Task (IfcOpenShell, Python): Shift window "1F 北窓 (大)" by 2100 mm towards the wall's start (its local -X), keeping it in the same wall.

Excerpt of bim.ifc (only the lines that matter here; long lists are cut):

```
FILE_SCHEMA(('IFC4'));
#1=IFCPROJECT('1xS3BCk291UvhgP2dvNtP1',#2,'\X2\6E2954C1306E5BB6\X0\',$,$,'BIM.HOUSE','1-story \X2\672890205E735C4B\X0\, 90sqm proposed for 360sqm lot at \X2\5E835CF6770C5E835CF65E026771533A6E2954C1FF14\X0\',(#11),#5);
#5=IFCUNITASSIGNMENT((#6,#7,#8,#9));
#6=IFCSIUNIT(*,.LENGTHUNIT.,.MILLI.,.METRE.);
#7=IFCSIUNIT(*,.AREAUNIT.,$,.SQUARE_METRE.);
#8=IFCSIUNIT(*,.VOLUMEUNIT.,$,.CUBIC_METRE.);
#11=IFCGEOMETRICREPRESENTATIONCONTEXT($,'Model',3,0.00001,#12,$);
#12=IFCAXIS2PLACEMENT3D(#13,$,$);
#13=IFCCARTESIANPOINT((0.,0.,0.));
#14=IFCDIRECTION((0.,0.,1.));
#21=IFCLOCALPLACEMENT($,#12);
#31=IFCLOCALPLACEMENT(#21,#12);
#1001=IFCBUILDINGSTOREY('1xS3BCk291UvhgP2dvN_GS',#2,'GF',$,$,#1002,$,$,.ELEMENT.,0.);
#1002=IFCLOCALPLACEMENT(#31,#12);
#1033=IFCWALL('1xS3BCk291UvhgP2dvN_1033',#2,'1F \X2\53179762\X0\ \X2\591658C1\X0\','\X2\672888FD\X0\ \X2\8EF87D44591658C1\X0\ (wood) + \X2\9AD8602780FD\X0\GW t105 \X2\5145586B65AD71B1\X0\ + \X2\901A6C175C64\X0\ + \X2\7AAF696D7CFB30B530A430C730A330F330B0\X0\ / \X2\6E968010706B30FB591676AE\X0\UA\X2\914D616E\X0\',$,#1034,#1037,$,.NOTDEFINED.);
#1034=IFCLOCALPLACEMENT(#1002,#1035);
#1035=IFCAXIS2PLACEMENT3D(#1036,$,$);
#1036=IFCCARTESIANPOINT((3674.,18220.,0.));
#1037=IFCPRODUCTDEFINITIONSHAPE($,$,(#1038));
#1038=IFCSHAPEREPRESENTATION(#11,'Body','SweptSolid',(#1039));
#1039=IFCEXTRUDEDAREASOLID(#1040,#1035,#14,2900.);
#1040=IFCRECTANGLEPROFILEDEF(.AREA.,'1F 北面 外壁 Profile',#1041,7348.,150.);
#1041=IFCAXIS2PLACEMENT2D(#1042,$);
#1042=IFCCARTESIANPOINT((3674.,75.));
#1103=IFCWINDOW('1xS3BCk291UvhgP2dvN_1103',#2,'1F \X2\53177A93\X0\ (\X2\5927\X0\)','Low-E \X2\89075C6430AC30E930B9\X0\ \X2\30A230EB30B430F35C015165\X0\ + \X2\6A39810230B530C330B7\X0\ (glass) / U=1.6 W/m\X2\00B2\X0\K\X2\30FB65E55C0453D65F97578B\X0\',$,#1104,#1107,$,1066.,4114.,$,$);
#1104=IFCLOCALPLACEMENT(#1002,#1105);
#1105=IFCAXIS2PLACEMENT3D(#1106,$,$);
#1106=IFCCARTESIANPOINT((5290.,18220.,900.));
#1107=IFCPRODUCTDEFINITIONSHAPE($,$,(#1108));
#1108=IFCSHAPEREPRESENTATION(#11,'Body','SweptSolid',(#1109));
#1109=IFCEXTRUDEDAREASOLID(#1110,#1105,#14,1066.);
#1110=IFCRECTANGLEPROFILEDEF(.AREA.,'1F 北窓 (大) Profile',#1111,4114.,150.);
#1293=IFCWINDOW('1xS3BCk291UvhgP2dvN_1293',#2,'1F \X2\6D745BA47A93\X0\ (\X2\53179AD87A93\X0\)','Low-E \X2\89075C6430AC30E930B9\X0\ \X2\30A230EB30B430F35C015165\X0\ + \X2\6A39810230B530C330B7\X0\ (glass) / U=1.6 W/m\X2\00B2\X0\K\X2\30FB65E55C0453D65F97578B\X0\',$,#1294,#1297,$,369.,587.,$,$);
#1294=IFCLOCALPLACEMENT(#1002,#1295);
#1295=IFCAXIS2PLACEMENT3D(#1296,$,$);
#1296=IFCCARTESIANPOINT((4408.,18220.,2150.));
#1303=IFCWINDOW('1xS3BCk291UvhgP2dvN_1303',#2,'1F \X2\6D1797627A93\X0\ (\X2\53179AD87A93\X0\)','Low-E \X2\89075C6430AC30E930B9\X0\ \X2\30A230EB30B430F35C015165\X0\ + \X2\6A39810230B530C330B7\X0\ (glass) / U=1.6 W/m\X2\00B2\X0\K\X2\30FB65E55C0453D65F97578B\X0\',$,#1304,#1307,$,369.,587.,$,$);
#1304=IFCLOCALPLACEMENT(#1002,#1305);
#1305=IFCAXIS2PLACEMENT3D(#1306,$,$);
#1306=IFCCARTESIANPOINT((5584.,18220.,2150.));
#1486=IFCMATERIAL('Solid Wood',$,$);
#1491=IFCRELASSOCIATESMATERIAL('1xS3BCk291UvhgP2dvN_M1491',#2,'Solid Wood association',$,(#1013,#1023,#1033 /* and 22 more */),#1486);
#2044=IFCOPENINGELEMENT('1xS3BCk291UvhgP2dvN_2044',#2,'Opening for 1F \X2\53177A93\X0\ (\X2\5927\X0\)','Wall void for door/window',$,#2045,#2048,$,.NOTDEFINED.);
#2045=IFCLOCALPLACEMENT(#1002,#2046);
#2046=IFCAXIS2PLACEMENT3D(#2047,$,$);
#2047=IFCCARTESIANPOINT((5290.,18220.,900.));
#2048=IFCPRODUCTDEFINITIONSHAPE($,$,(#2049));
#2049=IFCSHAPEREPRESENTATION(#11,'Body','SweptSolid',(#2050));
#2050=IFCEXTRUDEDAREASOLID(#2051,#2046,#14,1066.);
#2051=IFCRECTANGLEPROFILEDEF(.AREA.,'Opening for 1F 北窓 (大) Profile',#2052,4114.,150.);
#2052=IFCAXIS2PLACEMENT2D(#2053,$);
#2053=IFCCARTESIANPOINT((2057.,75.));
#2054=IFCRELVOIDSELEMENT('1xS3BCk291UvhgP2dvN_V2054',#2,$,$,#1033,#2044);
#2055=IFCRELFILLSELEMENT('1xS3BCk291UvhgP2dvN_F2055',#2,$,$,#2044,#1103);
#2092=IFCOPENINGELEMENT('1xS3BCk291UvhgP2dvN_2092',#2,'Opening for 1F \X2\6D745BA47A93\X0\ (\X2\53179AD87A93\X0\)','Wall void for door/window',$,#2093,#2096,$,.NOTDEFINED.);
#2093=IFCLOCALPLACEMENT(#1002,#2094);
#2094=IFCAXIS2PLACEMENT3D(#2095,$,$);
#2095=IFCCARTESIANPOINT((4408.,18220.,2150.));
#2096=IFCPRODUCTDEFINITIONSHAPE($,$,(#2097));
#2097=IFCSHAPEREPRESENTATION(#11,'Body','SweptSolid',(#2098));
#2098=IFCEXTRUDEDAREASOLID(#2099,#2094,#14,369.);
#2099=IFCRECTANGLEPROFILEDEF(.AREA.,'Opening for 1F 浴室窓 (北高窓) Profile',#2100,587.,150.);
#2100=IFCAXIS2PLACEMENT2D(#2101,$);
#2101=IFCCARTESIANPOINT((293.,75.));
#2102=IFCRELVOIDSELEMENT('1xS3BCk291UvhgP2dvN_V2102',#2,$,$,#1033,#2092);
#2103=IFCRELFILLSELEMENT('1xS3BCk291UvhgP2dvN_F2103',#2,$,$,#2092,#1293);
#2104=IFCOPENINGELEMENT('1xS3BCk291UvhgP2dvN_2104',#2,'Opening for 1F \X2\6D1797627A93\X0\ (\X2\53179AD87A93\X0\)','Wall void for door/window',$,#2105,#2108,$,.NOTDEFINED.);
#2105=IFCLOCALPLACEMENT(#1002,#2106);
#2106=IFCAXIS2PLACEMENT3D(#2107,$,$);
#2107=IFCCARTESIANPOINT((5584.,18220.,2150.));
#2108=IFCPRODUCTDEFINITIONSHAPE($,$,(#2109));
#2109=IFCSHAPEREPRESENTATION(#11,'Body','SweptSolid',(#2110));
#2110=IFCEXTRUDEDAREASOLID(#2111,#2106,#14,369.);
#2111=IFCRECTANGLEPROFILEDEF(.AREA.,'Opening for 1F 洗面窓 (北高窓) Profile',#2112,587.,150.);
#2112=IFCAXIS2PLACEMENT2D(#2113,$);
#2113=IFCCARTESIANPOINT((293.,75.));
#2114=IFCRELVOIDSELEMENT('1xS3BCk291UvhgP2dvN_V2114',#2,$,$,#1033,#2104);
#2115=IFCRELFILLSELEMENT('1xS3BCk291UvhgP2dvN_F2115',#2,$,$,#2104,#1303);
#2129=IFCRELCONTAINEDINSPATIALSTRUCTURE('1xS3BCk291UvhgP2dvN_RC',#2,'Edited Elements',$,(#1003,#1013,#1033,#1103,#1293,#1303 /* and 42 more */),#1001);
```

```python
import ifcopenshell
import ifcopenshell.api.geometry
import ifcopenshell.util.placement
import ifcopenshell.util.unit

model = ifcopenshell.open("bim.ifc")
unit_scale = ifcopenshell.util.unit.calculate_unit_scale(model)

window = model.by_guid("1xS3BCk291UvhgP2dvN_1103")
opening = window.FillsVoids[0].RelatingOpeningElement
wall = opening.VoidsElements[0].RelatingBuildingElement

wall_matrix = ifcopenshell.util.placement.get_local_placement(wall.ObjectPlacement)
shift = wall_matrix[:3, 0] * -2.1 / unit_scale
before = ifcopenshell.util.placement.get_local_placement(window.ObjectPlacement)[:3, 3].copy()

# The window is not placed relative to its opening, so move both.
for product in (opening, window):
    matrix = ifcopenshell.util.placement.get_local_placement(product.ObjectPlacement)
    matrix[:3, 3] += shift
    ifcopenshell.api.geometry.edit_object_placement(model, product=product, matrix=matrix, is_si=False)

after = ifcopenshell.util.placement.get_local_placement(window.ObjectPlacement)[:3, 3]
print("window moved by", (after - before).round(3) + 0.0)

model.write("bim_v2.ifc")
```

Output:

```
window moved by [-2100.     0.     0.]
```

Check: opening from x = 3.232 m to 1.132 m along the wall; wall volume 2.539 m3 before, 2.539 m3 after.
